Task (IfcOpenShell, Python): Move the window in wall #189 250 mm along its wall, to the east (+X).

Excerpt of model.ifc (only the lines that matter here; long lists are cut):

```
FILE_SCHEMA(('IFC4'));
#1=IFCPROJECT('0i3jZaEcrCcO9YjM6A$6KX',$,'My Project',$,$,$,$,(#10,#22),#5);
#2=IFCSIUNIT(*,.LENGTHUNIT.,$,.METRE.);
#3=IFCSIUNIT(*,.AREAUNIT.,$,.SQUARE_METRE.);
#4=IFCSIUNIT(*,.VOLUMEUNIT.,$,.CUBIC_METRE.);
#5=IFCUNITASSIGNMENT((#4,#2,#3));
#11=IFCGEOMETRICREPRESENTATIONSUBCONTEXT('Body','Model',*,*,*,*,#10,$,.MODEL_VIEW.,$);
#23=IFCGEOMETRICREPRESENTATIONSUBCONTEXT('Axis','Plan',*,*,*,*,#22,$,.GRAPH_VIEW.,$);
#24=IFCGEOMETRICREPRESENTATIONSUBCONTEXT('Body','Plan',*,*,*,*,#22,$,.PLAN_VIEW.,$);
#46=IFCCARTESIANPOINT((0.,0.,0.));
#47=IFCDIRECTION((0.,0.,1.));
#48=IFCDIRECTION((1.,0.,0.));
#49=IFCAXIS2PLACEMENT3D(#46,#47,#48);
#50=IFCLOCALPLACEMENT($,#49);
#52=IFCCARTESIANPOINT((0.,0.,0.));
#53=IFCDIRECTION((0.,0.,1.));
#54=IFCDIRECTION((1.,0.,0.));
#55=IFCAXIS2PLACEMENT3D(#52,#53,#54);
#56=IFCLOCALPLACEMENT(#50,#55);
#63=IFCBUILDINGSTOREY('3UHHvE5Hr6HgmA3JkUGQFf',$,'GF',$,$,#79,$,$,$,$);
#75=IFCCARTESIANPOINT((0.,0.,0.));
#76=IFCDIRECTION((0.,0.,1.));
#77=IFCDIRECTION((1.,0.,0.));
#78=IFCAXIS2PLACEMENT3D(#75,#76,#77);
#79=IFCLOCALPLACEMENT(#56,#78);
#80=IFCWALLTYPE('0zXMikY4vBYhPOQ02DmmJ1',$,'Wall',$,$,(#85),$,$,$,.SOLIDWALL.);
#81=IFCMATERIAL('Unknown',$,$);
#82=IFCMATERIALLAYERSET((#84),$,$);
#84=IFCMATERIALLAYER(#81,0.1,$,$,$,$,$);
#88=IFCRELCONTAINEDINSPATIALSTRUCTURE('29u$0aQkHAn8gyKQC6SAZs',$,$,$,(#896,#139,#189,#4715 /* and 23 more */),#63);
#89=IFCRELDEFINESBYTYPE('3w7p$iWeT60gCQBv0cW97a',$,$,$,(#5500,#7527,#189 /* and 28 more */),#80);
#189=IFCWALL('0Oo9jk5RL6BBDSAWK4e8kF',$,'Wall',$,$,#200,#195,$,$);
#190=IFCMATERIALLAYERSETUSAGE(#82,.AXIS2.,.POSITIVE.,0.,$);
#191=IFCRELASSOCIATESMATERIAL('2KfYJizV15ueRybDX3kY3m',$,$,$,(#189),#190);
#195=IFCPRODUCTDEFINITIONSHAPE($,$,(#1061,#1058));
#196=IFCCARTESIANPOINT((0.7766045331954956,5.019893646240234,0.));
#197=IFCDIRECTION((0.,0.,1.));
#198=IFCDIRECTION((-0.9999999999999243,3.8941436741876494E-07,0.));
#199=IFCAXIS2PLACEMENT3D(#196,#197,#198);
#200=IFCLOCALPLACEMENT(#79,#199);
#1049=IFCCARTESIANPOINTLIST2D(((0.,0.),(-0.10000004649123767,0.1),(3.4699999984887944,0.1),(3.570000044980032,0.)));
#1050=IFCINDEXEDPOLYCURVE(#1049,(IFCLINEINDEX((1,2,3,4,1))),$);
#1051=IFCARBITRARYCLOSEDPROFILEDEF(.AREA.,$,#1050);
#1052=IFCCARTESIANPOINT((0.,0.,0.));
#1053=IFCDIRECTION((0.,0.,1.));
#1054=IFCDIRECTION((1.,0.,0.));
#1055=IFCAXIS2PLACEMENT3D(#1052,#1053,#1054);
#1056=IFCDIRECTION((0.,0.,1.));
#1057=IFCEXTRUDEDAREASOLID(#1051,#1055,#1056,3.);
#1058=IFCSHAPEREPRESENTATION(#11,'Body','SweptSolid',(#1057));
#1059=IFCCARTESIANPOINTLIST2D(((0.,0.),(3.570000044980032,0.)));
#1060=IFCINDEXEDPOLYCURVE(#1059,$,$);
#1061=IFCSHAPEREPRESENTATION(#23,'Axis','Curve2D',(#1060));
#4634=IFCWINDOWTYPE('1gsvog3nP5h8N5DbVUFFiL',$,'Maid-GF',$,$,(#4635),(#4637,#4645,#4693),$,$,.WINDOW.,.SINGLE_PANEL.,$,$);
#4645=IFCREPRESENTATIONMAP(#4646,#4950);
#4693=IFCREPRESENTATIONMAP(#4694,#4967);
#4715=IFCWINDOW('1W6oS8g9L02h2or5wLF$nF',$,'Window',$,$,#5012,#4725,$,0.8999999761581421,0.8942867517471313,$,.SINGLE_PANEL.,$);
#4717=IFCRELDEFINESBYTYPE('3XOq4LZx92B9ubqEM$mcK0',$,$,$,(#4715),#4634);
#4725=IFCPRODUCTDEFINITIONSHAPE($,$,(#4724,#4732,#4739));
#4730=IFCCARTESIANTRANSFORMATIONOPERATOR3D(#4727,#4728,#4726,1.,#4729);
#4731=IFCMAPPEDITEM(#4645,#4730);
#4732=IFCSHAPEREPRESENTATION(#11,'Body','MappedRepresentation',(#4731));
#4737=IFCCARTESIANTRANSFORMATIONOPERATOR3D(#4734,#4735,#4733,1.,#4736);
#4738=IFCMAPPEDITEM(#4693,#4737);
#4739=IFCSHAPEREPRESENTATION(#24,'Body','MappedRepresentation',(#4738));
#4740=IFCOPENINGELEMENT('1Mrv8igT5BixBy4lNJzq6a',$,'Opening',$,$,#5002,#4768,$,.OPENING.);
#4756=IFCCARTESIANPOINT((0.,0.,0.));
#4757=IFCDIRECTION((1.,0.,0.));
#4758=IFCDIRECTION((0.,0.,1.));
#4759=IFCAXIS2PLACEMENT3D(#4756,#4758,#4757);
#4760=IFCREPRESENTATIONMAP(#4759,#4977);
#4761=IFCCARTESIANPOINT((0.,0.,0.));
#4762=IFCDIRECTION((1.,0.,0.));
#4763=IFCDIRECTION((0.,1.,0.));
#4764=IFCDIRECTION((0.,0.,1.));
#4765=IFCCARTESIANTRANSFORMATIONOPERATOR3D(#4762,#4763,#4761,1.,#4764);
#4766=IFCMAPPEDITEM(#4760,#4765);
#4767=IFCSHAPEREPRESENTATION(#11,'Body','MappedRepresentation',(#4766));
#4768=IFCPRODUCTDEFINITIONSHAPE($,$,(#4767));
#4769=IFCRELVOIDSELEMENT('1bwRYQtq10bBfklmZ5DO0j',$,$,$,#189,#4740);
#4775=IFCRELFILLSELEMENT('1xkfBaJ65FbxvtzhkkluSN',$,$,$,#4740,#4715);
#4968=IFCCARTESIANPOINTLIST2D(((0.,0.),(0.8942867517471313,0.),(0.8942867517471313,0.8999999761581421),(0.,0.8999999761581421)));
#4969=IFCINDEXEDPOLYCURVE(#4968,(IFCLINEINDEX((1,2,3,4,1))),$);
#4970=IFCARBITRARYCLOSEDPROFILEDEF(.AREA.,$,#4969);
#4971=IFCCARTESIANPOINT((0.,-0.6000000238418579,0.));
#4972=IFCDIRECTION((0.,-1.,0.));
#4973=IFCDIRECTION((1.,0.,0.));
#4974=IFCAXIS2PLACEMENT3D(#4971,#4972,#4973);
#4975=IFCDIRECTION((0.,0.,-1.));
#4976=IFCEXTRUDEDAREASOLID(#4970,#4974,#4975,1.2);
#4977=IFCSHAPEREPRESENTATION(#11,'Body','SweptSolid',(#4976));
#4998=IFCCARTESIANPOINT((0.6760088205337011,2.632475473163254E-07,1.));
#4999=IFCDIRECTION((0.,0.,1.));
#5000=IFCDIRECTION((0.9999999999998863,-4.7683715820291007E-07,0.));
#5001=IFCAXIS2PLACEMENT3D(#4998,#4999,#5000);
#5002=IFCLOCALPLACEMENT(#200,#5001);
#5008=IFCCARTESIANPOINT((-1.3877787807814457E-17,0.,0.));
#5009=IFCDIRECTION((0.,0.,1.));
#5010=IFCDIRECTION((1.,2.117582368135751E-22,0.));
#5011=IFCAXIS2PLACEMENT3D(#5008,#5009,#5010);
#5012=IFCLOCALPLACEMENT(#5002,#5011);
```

```python
import ifcopenshell
import ifcopenshell.api.geometry
import ifcopenshell.util.placement
import ifcopenshell.util.unit

model = ifcopenshell.open("model.ifc")
unit_scale = ifcopenshell.util.unit.calculate_unit_scale(model)

window = model.by_guid("1W6oS8g9L02h2or5wLF$nF")
opening = window.FillsVoids[0].RelatingOpeningElement
wall = opening.VoidsElements[0].RelatingBuildingElement

wall_matrix = ifcopenshell.util.placement.get_local_placement(wall.ObjectPlacement)
shift = wall_matrix[:3, 0] * -0.25 / unit_scale
before = ifcopenshell.util.placement.get_local_placement(window.ObjectPlacement)[:3, 3].copy()

# The window is placed relative to its opening, so it follows when the opening moves.
matrix = ifcopenshell.util.placement.get_local_placement(opening.ObjectPlacement)
matrix[:3, 3] += shift
ifcopenshell.api.geometry.edit_object_placement(
    model, product=opening, matrix=matrix, is_si=False, should_transform_children=True
)

after = ifcopenshell.util.placement.get_local_placement(window.ObjectPlacement)[:3, 3]
print("window moved by", (after - before).round(3) + 0.0)

model.write("model_v2.ifc")
```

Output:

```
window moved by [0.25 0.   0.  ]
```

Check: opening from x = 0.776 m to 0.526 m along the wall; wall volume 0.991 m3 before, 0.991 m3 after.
